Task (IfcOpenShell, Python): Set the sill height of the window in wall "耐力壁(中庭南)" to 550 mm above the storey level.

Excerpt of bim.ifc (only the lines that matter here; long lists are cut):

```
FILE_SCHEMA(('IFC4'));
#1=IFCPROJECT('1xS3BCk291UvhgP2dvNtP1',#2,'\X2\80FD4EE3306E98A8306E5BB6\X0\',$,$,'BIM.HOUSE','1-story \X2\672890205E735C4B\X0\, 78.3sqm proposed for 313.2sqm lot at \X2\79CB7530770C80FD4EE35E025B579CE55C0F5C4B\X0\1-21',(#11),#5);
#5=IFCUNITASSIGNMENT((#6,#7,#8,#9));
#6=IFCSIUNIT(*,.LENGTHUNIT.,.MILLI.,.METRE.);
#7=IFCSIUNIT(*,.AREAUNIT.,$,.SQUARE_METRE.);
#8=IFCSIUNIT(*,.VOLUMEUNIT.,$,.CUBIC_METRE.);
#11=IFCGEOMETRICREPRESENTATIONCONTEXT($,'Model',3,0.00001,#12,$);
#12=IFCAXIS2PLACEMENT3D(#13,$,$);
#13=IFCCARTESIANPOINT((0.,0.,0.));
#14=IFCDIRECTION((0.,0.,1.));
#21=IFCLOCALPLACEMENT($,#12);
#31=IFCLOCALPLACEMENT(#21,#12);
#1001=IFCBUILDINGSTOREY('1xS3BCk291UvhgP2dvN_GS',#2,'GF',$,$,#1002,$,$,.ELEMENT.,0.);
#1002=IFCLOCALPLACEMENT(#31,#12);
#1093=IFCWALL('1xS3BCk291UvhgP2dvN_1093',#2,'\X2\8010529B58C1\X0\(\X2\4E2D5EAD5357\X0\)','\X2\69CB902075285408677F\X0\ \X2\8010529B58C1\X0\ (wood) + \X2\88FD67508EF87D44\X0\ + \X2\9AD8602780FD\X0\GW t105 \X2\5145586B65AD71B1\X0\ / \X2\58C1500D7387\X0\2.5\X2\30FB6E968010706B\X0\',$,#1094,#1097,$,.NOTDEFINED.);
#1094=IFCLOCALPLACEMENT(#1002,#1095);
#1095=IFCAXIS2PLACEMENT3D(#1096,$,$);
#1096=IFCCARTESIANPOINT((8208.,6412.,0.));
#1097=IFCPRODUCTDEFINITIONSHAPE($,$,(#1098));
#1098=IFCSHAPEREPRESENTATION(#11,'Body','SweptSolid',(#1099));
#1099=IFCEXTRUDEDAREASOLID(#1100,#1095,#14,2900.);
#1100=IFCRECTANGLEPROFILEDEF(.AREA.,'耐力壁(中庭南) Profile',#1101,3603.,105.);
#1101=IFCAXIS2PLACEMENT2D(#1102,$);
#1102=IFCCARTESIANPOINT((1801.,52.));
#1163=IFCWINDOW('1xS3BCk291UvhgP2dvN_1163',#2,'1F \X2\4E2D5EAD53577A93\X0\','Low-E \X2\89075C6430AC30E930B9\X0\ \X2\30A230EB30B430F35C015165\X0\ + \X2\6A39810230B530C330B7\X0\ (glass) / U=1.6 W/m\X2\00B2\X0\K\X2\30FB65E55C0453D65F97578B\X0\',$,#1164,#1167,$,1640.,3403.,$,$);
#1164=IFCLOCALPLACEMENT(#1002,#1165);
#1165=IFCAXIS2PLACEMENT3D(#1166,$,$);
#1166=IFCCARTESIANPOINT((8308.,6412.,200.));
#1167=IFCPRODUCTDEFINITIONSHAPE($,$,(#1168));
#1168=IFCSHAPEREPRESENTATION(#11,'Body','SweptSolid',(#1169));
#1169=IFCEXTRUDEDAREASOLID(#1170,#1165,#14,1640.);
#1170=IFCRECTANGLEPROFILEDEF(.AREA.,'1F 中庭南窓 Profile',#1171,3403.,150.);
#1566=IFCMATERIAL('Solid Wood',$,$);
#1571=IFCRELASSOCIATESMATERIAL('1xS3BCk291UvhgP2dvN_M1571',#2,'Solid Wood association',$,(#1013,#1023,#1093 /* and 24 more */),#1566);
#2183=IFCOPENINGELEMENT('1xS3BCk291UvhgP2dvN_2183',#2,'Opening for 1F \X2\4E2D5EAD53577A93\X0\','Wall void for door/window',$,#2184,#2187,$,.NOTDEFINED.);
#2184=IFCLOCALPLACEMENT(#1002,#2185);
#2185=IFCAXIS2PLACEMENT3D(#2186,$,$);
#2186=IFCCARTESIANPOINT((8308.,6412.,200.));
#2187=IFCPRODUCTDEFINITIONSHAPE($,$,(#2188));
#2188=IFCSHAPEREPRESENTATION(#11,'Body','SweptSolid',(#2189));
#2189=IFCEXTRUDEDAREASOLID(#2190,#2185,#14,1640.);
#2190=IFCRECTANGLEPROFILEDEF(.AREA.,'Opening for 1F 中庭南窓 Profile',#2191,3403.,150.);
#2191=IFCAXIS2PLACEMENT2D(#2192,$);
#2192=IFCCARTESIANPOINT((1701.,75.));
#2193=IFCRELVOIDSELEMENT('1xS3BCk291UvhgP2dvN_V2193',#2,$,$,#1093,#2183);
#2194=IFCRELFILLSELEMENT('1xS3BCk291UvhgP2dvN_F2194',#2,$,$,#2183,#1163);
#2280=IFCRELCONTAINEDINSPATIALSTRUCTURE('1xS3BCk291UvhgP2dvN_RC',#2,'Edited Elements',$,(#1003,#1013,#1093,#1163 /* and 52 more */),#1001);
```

```python
import numpy as np
import ifcopenshell
import ifcopenshell.api.geometry
import ifcopenshell.geom
import ifcopenshell.util.element
import ifcopenshell.util.placement
import ifcopenshell.util.shape
import ifcopenshell.util.unit

model = ifcopenshell.open("bim.ifc")
unit_scale = ifcopenshell.util.unit.calculate_unit_scale(model)

window = model.by_id(1163)
opening = window.FillsVoids[0].RelatingOpeningElement
storey = ifcopenshell.util.element.get_container(window, ifc_class="IfcBuildingStorey")
level = ifcopenshell.util.placement.get_local_placement(storey.ObjectPlacement)[2, 3]

# The opening's origin need not be at the sill, so measure its lowest point.
shape = ifcopenshell.geom.create_shape(ifcopenshell.geom.settings(), opening)
bottom = ifcopenshell.util.shape.get_shape_bottom_elevation(shape, shape.geometry) / unit_scale
dz = level + 0.55 / unit_scale - bottom

shift = np.array([0.0, 0.0, dz])
# The window is not placed relative to its opening, so move both.
for product in (opening, window):
    matrix = ifcopenshell.util.placement.get_local_placement(product.ObjectPlacement)
    matrix[:3, 3] += shift
    ifcopenshell.api.geometry.edit_object_placement(model, product=product, matrix=matrix, is_si=False)

print(f"moved by {dz * unit_scale:+.3f} m")

model.write("bim_v2.ifc")
```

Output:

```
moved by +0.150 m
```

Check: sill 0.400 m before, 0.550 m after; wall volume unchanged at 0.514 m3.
